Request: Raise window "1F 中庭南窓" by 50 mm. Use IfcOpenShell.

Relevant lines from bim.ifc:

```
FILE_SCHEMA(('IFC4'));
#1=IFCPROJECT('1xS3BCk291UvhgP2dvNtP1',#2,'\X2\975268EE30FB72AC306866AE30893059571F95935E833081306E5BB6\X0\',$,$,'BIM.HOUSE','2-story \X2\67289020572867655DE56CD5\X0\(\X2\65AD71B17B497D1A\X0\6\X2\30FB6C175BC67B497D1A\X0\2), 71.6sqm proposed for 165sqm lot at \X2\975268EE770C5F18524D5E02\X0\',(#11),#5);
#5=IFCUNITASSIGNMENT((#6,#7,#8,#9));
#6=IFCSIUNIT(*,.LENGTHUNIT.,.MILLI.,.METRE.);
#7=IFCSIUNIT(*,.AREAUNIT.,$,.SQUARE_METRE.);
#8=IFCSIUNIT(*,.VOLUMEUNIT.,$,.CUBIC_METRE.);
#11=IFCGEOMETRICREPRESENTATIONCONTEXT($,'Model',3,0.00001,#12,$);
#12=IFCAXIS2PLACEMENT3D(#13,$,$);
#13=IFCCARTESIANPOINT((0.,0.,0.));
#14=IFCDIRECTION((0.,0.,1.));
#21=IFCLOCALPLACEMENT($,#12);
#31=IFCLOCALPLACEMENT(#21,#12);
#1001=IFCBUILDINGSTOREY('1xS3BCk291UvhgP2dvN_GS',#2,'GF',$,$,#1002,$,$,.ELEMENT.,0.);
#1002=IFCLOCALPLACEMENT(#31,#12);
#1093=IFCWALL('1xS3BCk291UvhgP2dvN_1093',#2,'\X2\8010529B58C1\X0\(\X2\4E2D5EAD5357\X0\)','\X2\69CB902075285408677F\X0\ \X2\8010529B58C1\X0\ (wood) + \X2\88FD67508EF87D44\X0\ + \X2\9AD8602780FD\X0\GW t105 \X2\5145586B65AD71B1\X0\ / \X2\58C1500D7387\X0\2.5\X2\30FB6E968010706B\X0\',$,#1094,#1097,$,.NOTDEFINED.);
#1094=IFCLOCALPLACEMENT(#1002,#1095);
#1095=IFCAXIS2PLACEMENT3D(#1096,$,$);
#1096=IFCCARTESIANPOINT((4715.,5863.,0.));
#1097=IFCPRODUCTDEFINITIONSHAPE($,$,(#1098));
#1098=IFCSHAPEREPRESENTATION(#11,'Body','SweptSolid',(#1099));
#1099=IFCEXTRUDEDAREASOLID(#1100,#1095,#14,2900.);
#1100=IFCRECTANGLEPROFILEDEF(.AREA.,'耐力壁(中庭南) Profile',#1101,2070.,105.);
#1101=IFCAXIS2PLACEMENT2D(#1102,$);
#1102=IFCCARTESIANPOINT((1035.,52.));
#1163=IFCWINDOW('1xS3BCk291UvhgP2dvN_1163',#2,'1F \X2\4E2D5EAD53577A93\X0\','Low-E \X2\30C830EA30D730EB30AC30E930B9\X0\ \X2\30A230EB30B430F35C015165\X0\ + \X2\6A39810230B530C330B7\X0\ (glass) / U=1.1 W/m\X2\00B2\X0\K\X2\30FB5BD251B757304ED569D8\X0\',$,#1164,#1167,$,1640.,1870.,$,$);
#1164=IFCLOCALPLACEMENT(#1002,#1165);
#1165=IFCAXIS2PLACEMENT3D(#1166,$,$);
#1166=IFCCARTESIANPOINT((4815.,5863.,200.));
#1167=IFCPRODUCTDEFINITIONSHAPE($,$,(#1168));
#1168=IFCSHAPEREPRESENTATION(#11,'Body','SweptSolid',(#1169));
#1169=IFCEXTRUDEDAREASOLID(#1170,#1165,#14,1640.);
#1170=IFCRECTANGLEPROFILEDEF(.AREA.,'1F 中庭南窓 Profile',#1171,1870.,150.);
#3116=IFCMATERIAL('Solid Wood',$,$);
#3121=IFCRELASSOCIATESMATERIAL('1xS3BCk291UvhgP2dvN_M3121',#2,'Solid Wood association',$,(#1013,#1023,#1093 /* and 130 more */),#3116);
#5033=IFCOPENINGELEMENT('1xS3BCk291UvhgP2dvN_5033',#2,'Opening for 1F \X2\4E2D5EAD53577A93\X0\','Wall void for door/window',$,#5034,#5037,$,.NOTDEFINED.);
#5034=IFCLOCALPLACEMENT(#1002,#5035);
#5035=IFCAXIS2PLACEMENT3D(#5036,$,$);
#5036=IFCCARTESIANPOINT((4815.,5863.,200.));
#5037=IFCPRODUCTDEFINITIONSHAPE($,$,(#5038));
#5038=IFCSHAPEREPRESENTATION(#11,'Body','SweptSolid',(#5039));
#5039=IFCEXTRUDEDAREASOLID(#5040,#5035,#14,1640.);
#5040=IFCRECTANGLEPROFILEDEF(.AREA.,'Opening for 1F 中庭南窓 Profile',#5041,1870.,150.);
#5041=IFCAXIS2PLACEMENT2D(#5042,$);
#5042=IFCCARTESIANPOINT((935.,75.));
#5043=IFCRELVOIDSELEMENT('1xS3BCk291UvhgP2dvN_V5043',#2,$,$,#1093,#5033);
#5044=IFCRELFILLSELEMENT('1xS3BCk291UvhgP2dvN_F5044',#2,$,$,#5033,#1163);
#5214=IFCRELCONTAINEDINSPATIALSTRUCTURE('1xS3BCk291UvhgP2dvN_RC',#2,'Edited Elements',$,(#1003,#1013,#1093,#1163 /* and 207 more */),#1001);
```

```python
import numpy as np
import ifcopenshell
import ifcopenshell.api.geometry
import ifcopenshell.util.placement
import ifcopenshell.util.unit

model = ifcopenshell.open("bim.ifc")
unit_scale = ifcopenshell.util.unit.calculate_unit_scale(model)

window = model.by_guid("1xS3BCk291UvhgP2dvN_1163")
opening = window.FillsVoids[0].RelatingOpeningElement
dz = 50.0

shift = np.array([0.0, 0.0, dz])
# The window is not placed relative to its opening, so move both.
for product in (opening, window):
    matrix = ifcopenshell.util.placement.get_local_placement(product.ObjectPlacement)
    matrix[:3, 3] += shift
    ifcopenshell.api.geometry.edit_object_placement(model, product=product, matrix=matrix, is_si=False)

print(f"moved by {dz * unit_scale:+.3f} m")

model.write("bim_edited.ifc")
```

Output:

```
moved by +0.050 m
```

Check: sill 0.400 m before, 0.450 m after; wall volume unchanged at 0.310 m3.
